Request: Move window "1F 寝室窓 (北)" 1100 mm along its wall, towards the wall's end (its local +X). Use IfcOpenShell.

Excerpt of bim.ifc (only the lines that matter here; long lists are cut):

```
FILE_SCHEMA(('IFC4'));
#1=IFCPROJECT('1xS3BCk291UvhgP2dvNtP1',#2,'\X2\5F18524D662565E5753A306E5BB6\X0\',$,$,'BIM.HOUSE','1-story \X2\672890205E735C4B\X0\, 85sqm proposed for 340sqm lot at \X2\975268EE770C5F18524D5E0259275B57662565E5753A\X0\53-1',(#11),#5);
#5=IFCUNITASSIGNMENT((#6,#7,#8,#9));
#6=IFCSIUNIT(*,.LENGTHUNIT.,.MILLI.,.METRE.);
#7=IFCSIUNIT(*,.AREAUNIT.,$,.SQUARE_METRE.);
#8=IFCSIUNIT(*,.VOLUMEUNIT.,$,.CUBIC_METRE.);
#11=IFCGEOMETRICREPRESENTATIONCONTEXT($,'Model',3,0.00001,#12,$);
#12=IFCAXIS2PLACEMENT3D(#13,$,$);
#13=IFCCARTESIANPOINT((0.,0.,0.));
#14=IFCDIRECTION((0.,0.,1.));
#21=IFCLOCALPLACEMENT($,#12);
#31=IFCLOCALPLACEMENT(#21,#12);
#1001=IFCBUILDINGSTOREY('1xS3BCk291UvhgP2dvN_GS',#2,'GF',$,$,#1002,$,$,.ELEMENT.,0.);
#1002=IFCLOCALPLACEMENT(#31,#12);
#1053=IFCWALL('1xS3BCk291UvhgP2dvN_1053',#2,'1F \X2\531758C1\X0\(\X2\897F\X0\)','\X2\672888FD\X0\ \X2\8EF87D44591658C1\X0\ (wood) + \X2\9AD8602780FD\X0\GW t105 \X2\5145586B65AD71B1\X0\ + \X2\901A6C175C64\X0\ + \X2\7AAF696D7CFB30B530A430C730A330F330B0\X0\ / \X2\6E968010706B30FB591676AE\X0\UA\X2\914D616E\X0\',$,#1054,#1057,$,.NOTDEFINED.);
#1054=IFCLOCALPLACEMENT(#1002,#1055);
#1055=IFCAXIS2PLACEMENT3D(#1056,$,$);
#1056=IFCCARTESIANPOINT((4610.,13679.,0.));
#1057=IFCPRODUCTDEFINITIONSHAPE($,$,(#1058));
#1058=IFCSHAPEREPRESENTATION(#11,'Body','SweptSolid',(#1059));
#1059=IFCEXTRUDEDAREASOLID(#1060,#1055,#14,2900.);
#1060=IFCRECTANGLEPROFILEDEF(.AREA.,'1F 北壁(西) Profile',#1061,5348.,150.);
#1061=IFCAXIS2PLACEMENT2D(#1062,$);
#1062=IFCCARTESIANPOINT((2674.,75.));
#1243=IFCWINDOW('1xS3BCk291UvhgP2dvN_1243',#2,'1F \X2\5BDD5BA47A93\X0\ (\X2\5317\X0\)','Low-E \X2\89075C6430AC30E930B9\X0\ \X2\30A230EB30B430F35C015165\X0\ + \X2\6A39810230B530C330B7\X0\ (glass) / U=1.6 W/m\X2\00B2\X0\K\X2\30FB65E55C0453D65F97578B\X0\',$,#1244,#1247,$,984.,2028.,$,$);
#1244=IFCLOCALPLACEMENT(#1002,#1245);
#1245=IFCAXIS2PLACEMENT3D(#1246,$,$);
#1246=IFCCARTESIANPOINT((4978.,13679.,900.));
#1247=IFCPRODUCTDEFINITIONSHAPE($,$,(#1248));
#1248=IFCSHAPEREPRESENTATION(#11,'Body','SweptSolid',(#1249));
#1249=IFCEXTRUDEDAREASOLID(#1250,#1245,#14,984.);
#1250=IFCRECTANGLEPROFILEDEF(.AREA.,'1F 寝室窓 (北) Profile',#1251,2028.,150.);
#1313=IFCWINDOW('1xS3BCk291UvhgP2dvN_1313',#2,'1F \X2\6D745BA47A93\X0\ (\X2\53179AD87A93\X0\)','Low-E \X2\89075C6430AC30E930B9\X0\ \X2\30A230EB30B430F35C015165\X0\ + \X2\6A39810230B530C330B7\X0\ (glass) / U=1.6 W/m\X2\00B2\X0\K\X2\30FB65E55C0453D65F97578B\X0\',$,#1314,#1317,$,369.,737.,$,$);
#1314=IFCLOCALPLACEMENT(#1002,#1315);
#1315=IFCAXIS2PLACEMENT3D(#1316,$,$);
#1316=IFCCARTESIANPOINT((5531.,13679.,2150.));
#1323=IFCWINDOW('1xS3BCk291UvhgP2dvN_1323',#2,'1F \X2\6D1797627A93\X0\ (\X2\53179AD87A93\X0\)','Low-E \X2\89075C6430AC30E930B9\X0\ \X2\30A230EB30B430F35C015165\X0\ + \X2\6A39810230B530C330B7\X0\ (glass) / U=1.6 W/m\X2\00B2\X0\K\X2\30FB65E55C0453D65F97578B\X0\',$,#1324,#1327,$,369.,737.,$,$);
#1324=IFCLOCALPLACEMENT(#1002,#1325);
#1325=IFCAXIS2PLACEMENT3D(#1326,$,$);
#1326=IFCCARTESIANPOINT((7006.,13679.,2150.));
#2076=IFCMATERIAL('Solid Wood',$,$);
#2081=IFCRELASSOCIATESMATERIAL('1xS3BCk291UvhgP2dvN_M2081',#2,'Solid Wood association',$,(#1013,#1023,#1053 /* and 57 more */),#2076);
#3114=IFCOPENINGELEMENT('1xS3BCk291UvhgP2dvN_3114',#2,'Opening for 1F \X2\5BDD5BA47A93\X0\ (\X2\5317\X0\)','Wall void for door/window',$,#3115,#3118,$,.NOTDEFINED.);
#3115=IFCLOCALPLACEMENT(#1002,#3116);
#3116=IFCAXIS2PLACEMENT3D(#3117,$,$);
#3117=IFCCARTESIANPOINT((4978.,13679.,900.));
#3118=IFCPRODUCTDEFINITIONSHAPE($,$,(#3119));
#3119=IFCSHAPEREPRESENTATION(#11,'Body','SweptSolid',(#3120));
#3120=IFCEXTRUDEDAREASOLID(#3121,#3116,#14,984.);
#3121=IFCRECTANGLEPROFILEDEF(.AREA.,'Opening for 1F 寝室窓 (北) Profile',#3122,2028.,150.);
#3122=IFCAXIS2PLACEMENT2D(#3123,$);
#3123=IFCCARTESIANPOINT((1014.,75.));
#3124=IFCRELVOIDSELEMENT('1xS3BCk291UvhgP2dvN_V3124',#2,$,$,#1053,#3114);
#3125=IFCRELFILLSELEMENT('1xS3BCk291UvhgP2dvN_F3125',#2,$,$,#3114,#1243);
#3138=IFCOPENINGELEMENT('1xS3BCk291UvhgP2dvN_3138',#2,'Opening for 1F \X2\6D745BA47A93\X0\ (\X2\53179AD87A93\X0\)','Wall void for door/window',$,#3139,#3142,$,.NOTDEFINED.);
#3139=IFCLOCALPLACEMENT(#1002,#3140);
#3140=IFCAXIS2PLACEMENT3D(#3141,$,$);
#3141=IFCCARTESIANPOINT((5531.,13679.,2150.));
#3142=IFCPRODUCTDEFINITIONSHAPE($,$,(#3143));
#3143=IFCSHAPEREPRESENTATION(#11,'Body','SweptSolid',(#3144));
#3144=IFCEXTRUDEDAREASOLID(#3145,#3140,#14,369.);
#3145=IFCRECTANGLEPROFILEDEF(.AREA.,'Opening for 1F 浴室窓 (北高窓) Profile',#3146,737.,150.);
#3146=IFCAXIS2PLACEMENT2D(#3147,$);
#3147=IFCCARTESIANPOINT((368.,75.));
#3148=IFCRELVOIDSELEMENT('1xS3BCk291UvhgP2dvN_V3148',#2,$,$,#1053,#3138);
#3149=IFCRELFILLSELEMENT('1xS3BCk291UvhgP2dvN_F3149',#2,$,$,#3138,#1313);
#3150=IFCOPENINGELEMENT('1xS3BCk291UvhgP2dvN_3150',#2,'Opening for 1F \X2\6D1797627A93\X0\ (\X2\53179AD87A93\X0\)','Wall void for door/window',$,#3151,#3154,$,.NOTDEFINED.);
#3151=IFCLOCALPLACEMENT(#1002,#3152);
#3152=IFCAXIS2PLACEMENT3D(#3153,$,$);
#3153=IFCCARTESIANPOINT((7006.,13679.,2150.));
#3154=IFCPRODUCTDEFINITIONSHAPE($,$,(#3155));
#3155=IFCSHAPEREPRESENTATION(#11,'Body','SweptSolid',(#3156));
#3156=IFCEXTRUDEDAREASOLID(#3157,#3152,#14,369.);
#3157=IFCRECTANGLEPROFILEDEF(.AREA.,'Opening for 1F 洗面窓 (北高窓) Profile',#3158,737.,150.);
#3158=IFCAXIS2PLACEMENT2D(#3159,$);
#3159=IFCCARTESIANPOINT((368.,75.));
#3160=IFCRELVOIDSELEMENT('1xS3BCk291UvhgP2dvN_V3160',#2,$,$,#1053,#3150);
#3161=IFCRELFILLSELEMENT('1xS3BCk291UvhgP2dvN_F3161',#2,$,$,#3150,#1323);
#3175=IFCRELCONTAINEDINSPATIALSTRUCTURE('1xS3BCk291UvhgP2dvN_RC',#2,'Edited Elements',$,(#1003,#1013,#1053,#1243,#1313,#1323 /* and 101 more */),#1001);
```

```python
import ifcopenshell
import ifcopenshell.api.geometry
import ifcopenshell.util.placement
import ifcopenshell.util.unit

model = ifcopenshell.open("bim.ifc")
unit_scale = ifcopenshell.util.unit.calculate_unit_scale(model)

window = model.by_id(1243)
opening = window.FillsVoids[0].RelatingOpeningElement
wall = opening.VoidsElements[0].RelatingBuildingElement

wall_matrix = ifcopenshell.util.placement.get_local_placement(wall.ObjectPlacement)
shift = wall_matrix[:3, 0] * 1.1 / unit_scale
before = ifcopenshell.util.placement.get_local_placement(window.ObjectPlacement)[:3, 3].copy()

# The window is not placed relative to its opening, so move both.
for product in (opening, window):
    matrix = ifcopenshell.util.placement.get_local_placement(product.ObjectPlacement)
    matrix[:3, 3] += shift
    ifcopenshell.api.geometry.edit_object_placement(model, product=product, matrix=matrix, is_si=False)

after = ifcopenshell.util.placement.get_local_placement(window.ObjectPlacement)[:3, 3]
print("window moved by", (after - before).round(3) + 0.0)

model.write("bim-out.ifc")
```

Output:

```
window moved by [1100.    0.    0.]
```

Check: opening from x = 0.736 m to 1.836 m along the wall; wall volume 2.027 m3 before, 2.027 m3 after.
